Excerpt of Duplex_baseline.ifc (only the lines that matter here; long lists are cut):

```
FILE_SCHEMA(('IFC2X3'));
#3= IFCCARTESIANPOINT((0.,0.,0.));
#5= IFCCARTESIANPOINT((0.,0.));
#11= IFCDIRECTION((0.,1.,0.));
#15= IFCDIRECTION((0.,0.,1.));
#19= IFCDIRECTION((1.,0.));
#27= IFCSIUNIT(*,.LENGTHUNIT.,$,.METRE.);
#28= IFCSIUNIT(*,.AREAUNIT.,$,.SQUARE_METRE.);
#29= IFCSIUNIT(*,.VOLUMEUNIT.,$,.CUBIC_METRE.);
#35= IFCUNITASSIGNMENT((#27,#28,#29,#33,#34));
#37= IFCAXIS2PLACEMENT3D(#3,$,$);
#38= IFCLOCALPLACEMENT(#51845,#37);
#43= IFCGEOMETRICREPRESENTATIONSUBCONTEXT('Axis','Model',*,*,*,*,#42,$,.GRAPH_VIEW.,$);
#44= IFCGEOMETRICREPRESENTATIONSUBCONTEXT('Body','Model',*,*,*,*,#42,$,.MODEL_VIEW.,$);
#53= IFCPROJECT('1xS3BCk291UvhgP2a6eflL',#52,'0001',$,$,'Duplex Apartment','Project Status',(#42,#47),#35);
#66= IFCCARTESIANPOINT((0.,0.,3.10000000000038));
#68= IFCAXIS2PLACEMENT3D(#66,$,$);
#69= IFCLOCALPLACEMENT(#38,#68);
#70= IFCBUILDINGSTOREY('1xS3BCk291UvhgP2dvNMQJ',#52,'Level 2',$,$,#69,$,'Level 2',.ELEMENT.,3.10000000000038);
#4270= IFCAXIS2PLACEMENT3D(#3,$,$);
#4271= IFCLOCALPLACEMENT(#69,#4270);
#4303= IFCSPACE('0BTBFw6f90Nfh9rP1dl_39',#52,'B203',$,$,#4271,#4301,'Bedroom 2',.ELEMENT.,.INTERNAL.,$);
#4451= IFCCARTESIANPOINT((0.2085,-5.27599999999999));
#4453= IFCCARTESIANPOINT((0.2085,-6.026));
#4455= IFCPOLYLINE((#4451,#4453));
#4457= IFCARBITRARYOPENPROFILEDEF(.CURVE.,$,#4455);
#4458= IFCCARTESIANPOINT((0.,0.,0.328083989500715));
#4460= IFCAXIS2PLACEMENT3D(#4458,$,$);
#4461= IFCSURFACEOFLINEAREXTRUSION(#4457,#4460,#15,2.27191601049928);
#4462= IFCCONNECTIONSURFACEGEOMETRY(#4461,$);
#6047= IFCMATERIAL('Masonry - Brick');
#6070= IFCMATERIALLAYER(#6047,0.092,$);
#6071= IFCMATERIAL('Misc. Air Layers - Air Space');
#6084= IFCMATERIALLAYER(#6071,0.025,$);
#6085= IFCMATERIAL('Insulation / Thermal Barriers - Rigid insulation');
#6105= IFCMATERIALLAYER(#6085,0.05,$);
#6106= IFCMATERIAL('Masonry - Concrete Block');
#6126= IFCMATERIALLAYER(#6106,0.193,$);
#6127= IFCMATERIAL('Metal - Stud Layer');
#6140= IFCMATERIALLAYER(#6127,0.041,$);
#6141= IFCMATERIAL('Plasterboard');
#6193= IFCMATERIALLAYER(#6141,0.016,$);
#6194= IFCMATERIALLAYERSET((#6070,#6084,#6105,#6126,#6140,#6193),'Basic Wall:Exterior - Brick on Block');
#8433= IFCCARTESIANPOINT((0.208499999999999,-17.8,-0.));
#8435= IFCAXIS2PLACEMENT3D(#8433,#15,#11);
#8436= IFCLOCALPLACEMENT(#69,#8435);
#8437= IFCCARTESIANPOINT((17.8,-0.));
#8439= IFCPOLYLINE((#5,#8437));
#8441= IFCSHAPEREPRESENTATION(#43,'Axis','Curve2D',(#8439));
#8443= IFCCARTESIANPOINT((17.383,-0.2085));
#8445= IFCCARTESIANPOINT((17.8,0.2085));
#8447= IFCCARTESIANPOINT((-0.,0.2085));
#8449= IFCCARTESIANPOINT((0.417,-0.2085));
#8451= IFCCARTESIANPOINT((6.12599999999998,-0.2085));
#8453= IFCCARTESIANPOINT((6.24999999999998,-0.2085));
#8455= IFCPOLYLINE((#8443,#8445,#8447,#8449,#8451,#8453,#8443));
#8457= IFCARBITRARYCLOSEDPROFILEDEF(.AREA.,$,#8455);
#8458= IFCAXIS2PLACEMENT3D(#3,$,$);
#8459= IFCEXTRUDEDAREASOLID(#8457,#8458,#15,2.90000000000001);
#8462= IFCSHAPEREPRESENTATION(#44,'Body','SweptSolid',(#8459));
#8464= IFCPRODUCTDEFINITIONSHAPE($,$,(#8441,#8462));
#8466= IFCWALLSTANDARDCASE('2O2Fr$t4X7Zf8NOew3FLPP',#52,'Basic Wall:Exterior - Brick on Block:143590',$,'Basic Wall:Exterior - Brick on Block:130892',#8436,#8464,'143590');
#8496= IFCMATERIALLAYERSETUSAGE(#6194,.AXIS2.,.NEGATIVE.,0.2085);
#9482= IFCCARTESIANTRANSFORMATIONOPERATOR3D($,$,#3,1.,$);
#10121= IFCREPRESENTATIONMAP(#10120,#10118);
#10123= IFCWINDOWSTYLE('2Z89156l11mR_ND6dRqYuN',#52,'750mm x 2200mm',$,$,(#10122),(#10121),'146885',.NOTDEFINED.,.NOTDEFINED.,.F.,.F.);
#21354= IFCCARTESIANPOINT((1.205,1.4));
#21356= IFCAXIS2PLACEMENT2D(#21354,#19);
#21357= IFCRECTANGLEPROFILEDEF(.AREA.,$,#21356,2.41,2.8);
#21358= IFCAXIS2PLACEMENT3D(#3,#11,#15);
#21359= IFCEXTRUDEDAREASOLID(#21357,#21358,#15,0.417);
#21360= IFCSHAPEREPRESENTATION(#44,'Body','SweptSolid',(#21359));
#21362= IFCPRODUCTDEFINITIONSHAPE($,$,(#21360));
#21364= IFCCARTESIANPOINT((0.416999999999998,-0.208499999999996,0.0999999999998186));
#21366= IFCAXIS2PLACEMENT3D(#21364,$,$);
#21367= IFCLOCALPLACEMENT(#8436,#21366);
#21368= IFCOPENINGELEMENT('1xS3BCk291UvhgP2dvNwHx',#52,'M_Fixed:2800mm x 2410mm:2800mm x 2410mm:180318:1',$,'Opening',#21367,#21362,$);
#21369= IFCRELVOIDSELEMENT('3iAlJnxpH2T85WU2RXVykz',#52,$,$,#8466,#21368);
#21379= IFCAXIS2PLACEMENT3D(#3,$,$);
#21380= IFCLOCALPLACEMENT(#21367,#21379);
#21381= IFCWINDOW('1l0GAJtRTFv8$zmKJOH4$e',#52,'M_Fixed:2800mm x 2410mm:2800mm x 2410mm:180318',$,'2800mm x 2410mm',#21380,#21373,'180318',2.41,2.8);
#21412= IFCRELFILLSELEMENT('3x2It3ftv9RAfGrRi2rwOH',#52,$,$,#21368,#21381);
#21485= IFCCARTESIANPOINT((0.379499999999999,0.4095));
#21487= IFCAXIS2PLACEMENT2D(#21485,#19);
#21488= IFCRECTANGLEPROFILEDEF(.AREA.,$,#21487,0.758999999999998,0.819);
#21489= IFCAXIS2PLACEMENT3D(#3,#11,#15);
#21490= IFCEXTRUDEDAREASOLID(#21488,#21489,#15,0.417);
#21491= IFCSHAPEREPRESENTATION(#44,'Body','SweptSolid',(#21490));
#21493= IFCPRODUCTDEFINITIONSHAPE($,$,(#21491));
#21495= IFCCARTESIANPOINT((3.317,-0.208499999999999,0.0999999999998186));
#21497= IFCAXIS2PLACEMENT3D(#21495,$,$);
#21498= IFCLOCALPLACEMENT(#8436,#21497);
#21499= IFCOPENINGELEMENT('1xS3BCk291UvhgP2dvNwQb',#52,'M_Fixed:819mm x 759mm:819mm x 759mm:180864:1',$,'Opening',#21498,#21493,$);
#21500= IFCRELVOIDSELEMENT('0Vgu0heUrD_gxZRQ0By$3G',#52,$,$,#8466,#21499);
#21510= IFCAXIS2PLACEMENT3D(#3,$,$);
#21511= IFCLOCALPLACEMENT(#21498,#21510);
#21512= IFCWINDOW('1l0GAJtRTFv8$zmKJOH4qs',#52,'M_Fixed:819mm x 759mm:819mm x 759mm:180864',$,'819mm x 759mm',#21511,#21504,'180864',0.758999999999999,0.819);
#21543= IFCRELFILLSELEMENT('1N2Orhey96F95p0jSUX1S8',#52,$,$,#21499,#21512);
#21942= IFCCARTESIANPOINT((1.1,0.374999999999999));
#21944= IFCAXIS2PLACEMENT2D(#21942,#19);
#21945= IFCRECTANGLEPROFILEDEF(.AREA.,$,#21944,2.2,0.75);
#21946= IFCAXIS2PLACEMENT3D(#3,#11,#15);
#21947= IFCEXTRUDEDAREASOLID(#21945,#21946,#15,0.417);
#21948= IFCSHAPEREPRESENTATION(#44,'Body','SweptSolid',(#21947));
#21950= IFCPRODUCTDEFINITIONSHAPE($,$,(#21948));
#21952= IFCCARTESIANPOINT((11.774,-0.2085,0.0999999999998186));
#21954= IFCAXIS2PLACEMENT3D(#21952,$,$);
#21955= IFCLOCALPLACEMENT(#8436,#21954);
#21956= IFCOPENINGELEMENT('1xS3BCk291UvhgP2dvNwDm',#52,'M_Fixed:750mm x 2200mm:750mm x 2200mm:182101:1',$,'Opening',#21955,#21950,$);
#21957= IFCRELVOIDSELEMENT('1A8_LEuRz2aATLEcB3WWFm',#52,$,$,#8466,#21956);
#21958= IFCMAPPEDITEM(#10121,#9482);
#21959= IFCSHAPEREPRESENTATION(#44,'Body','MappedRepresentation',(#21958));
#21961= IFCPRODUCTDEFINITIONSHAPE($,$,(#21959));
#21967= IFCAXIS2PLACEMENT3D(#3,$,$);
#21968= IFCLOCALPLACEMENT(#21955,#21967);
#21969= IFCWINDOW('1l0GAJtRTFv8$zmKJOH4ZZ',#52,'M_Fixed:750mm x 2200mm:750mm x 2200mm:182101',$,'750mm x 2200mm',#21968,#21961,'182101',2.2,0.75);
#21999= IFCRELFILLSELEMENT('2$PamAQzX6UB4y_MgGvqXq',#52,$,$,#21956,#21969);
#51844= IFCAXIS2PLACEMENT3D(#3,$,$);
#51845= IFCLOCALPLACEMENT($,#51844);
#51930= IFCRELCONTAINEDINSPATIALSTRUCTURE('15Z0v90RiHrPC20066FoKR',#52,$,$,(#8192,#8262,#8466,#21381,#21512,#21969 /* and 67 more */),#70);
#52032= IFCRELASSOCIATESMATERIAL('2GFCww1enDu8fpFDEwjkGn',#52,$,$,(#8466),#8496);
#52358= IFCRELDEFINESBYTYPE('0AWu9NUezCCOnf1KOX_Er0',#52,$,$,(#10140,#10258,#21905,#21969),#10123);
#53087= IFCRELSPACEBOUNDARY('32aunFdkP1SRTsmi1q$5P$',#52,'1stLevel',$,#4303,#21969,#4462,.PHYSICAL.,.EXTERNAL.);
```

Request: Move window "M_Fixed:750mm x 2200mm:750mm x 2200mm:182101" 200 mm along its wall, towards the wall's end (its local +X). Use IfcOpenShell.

```python
import numpy as np
import ifcopenshell
import ifcopenshell.api.geometry
import ifcopenshell.util.placement
import ifcopenshell.util.unit

model = ifcopenshell.open("Duplex_baseline.ifc")
unit_scale = ifcopenshell.util.unit.calculate_unit_scale(model)

window = model.by_guid("1l0GAJtRTFv8$zmKJOH4ZZ")
opening = window.FillsVoids[0].RelatingOpeningElement
wall = opening.VoidsElements[0].RelatingBuildingElement

wall_matrix = ifcopenshell.util.placement.get_local_placement(wall.ObjectPlacement)
shift = wall_matrix[:3, 0] * 0.2 / unit_scale
before = ifcopenshell.util.placement.get_local_placement(window.ObjectPlacement)[:3, 3].copy()

# The window is placed relative to its opening, so it follows when the opening moves.
matrix = ifcopenshell.util.placement.get_local_placement(opening.ObjectPlacement)
matrix[:3, 3] += shift
ifcopenshell.api.geometry.edit_object_placement(
    model, product=opening, matrix=matrix, is_si=False, should_transform_children=True
)

# Space boundary surfaces are stored in each space's coordinates; move them too.
for rel in window.ProvidesBoundaries:
    if not rel.ConnectionGeometry:
        continue
    surface = rel.ConnectionGeometry.SurfaceOnRelatingElement
    space_matrix = ifcopenshell.util.placement.get_local_placement(rel.RelatingSpace.ObjectPlacement)
    point = np.array(surface.Position.Location.Coordinates) + space_matrix[:3, :3].T @ shift
    surface.Position = model.createIfcAxis2Placement3D(
        model.createIfcCartesianPoint(point.tolist()), surface.Position.Axis, surface.Position.RefDirection
    )

after = ifcopenshell.util.placement.get_local_placement(window.ObjectPlacement)[:3, 3]
print("window moved by", (after - before).round(3) + 0.0)

model.write("Duplex_baseline_rev.ifc")
```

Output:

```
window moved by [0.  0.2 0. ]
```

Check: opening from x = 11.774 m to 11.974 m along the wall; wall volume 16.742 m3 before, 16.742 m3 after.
